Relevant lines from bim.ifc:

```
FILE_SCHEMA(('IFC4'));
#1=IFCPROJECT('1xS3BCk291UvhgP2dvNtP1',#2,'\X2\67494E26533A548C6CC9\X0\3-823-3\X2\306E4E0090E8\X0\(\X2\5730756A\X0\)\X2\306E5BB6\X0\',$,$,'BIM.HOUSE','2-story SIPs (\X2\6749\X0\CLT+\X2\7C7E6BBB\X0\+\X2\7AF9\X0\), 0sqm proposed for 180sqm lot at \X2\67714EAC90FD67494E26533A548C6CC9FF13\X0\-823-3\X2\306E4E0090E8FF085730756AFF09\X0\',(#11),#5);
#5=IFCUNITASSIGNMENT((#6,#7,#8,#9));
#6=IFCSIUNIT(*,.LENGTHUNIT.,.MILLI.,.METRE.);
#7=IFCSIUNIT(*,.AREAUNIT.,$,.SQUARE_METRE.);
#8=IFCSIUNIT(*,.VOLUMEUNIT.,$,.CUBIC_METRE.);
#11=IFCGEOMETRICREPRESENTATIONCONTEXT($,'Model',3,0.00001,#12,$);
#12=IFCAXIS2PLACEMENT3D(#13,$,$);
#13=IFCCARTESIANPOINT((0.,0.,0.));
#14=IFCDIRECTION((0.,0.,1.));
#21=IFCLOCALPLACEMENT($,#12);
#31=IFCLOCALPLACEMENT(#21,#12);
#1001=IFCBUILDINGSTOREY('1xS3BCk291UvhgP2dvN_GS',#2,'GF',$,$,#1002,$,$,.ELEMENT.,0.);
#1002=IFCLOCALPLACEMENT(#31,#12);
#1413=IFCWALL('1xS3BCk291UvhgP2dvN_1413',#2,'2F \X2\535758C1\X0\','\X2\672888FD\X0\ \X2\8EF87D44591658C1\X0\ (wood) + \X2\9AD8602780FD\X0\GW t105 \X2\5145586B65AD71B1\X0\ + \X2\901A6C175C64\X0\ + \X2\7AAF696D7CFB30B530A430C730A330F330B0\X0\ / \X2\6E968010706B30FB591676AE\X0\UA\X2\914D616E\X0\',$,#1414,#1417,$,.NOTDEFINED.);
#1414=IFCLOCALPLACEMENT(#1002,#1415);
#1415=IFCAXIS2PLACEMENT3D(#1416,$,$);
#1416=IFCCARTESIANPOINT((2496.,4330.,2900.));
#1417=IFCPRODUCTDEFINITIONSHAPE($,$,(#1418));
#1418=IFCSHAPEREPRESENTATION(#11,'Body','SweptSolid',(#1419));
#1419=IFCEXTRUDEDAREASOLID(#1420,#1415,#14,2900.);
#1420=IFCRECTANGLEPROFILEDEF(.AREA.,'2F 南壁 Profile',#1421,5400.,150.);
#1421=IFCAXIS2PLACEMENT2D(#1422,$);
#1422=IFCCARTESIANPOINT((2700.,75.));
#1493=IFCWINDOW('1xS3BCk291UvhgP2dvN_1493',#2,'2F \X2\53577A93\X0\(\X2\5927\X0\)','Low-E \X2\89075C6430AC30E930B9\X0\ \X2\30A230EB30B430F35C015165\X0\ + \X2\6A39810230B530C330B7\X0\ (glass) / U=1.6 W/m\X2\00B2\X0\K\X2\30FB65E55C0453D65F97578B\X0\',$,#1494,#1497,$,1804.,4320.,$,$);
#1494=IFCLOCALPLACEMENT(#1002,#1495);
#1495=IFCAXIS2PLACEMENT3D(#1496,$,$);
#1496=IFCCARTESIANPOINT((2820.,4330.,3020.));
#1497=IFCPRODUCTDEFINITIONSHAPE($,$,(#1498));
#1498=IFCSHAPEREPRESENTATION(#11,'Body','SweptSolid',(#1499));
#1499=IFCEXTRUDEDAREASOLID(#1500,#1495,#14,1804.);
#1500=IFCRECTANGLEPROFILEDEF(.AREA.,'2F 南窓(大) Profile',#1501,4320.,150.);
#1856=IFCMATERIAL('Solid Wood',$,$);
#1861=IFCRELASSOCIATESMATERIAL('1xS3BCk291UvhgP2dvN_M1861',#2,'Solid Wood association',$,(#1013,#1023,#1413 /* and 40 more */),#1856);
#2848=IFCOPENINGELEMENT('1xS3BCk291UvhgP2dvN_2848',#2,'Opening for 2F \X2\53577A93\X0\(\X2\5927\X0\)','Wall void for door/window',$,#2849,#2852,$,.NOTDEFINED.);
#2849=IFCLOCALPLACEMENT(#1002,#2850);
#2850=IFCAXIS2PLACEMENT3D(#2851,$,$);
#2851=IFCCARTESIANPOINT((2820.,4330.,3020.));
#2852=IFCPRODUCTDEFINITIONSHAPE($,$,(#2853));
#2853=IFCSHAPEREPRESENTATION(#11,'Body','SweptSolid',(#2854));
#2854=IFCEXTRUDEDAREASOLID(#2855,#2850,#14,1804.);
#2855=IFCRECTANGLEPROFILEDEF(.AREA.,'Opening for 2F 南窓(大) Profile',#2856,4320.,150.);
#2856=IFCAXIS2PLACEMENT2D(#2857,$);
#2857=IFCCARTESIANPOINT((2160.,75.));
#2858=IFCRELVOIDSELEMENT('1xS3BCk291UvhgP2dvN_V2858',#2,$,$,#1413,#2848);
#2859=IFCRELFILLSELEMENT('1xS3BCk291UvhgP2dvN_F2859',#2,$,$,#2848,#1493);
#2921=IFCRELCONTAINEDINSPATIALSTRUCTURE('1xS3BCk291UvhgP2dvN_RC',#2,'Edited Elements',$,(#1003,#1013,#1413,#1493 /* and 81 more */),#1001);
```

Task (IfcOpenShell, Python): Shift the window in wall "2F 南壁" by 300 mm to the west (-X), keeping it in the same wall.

```python
import ifcopenshell
import ifcopenshell.api.geometry
import ifcopenshell.util.placement
import ifcopenshell.util.unit

model = ifcopenshell.open("bim.ifc")
unit_scale = ifcopenshell.util.unit.calculate_unit_scale(model)

window = model.by_id(1493)
opening = window.FillsVoids[0].RelatingOpeningElement
wall = opening.VoidsElements[0].RelatingBuildingElement

wall_matrix = ifcopenshell.util.placement.get_local_placement(wall.ObjectPlacement)
shift = wall_matrix[:3, 0] * -0.3 / unit_scale
before = ifcopenshell.util.placement.get_local_placement(window.ObjectPlacement)[:3, 3].copy()

# The window is not placed relative to its opening, so move both.
for product in (opening, window):
    matrix = ifcopenshell.util.placement.get_local_placement(product.ObjectPlacement)
    matrix[:3, 3] += shift
    ifcopenshell.api.geometry.edit_object_placement(model, product=product, matrix=matrix, is_si=False)

after = ifcopenshell.util.placement.get_local_placement(window.ObjectPlacement)[:3, 3]
print("window moved by", (after - before).round(3) + 0.0)

model.write("bim_updated.ifc")
```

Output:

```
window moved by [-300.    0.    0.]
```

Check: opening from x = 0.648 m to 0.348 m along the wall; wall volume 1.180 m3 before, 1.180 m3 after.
